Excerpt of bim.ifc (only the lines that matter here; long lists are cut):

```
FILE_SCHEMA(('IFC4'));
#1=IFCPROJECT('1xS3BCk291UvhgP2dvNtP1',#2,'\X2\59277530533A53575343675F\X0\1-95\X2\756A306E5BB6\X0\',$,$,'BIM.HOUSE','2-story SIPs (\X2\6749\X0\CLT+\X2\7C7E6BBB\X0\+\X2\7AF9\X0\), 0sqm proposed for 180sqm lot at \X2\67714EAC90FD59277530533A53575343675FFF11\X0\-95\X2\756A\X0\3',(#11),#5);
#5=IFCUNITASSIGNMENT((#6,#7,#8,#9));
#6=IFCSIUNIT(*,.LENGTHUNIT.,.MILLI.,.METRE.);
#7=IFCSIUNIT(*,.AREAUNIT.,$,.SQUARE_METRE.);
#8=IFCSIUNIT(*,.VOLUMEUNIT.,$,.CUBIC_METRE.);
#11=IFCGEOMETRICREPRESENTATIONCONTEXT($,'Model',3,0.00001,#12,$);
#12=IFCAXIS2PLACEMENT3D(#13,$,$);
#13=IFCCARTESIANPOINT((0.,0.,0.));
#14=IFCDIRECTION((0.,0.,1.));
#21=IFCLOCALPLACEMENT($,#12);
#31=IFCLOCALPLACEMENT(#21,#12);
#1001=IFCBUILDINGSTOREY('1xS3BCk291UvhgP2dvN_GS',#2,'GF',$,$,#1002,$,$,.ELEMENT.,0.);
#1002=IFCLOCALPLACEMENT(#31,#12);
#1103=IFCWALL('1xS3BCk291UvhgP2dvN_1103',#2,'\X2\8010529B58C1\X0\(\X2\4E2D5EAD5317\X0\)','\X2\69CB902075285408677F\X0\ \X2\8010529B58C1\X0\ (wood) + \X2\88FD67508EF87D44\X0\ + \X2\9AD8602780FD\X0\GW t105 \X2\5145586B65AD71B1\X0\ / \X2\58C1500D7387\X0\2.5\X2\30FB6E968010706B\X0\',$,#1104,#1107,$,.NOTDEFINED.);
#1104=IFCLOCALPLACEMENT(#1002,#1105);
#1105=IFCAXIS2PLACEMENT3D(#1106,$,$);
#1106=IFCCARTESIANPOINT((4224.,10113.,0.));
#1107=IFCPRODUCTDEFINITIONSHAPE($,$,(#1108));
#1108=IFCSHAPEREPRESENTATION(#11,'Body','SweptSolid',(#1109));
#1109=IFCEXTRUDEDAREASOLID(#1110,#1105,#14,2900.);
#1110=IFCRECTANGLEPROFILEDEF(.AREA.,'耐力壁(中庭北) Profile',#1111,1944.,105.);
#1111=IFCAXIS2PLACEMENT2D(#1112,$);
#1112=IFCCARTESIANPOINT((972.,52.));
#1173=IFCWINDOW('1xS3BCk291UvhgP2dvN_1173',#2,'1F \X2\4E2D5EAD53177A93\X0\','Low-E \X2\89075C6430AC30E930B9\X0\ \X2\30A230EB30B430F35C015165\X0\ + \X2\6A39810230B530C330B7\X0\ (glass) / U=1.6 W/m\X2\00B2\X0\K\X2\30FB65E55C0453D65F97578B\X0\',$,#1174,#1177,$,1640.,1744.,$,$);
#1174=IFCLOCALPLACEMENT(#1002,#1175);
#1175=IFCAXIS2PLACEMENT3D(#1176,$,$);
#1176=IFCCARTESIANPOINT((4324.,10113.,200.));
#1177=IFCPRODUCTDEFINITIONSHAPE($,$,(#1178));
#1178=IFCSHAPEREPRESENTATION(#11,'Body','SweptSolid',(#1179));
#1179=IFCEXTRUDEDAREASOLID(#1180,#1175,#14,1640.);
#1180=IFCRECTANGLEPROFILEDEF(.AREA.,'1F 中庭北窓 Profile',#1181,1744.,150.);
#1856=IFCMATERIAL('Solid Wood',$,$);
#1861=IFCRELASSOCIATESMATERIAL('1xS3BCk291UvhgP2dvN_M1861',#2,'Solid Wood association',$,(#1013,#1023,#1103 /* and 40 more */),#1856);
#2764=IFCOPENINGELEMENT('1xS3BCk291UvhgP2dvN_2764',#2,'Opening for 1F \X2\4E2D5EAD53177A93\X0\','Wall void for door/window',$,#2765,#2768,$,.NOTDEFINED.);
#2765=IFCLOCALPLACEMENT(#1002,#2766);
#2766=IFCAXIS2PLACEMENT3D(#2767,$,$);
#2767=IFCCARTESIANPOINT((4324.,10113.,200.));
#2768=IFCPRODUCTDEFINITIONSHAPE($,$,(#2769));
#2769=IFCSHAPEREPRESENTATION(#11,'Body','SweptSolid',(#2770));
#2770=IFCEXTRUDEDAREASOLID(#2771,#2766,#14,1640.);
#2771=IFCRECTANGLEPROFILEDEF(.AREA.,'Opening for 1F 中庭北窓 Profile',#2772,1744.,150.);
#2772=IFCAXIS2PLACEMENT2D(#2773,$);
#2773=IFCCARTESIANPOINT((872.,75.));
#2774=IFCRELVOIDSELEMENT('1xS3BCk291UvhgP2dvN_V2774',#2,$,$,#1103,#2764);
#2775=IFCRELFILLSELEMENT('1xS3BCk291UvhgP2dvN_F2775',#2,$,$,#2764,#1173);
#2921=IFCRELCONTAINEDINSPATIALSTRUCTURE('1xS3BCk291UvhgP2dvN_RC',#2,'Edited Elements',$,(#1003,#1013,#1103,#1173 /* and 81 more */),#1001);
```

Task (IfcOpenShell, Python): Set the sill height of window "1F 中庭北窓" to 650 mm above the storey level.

```python
import numpy as np
import ifcopenshell
import ifcopenshell.api.geometry
import ifcopenshell.geom
import ifcopenshell.util.element
import ifcopenshell.util.placement
import ifcopenshell.util.shape
import ifcopenshell.util.unit

model = ifcopenshell.open("bim.ifc")
unit_scale = ifcopenshell.util.unit.calculate_unit_scale(model)

window = model.by_id(1173)
opening = window.FillsVoids[0].RelatingOpeningElement
storey = ifcopenshell.util.element.get_container(window, ifc_class="IfcBuildingStorey")
level = ifcopenshell.util.placement.get_local_placement(storey.ObjectPlacement)[2, 3]

# The opening's origin need not be at the sill, so measure its lowest point.
shape = ifcopenshell.geom.create_shape(ifcopenshell.geom.settings(), opening)
bottom = ifcopenshell.util.shape.get_shape_bottom_elevation(shape, shape.geometry) / unit_scale
dz = level + 650.0 - bottom

shift = np.array([0.0, 0.0, dz])
# The window is not placed relative to its opening, so move both.
for product in (opening, window):
    matrix = ifcopenshell.util.placement.get_local_placement(product.ObjectPlacement)
    matrix[:3, 3] += shift
    ifcopenshell.api.geometry.edit_object_placement(model, product=product, matrix=matrix, is_si=False)

print(f"moved by {dz * unit_scale:+.3f} m")

model.write("bim_edited.ifc")
```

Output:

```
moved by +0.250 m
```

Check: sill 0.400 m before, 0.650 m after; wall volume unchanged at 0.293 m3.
